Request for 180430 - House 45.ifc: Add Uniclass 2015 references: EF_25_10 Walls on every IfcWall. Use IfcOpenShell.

First a look at what the model holds.

```python
import ifcopenshell

model = ifcopenshell.open("180430 - House 45.ifc")
print(model.schema)
print("classifications:", [c.Name for c in model.by_type("IfcClassification")])
for ifc_class in ("IfcDoor", "IfcRoof", "IfcStair", "IfcWall", "IfcWindow"):
    print(ifc_class, len(model.by_type(ifc_class)))
```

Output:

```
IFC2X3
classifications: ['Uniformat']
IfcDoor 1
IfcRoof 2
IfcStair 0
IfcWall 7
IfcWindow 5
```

```python
import ifcopenshell
import ifcopenshell.api.classification

model = ifcopenshell.open("180430 - House 45.ifc")

# IFC2X3 requires Source and Edition and has no link from the project to the system.
system = model.create_entity("IfcClassification", Source="NBS", Edition="2015", Name="Uniclass 2015")

codes = {
    "IfcWall": ("EF_25_10", "Walls"),
}
for ifc_class, (code, name) in codes.items():
    products = model.by_type(ifc_class)
    ifcopenshell.api.classification.add_reference(
        model, products=products, classification=system, identification=code, name=name
    )
    print(code, len(products))

model.write("180430 - House 45_rev.ifc")
```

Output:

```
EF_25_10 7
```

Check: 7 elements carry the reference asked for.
